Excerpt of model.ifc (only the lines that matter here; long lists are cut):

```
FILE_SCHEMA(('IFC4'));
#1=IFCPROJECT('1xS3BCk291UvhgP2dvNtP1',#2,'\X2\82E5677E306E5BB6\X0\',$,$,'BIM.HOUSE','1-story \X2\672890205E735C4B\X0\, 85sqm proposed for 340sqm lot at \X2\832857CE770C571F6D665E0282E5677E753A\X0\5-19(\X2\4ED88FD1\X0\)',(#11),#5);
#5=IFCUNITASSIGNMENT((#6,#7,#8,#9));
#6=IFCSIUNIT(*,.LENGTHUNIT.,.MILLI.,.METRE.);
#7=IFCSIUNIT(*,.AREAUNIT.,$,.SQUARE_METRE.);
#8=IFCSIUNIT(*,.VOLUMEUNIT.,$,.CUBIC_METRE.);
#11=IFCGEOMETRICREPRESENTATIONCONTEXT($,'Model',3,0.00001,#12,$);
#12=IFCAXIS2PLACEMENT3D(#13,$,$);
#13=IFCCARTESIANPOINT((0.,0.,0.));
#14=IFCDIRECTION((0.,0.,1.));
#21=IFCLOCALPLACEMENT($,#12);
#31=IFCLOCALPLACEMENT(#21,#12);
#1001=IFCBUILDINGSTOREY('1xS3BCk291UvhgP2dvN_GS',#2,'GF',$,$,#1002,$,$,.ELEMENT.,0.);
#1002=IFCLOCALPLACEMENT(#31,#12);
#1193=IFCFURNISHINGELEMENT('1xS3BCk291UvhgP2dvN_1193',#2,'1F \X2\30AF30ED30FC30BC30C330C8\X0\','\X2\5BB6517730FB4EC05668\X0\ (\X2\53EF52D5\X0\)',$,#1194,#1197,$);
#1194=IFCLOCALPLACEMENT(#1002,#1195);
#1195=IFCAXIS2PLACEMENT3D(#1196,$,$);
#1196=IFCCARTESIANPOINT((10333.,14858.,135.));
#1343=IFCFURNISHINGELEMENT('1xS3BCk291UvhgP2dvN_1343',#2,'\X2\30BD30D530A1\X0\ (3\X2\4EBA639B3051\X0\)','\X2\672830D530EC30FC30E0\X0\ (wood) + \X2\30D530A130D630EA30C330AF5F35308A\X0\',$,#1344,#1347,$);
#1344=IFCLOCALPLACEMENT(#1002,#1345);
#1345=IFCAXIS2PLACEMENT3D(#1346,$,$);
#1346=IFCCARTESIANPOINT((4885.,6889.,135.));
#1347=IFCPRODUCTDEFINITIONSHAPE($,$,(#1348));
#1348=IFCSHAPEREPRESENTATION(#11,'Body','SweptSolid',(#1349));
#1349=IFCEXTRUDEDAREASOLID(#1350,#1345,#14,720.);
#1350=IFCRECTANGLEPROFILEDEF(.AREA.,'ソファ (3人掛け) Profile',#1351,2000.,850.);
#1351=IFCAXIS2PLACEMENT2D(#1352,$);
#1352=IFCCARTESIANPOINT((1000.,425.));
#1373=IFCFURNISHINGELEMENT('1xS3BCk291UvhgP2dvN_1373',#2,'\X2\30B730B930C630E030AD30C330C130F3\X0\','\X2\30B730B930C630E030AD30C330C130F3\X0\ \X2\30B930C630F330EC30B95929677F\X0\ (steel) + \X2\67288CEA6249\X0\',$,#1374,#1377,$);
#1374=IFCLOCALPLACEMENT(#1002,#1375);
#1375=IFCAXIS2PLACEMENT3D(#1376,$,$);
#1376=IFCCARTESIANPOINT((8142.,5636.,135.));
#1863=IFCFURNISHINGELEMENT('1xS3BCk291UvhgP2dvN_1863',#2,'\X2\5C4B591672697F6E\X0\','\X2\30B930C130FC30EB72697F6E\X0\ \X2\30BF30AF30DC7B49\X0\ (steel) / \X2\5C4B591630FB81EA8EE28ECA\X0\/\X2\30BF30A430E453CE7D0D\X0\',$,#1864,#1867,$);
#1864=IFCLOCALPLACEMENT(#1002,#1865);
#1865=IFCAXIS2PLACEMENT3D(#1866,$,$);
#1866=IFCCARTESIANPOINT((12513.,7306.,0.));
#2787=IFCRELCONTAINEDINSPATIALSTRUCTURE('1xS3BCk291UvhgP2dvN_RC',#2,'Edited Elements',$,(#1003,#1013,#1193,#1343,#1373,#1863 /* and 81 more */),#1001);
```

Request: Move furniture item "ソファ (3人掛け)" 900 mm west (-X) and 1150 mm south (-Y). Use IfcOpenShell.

```python
import ifcopenshell
import ifcopenshell.api.geometry
import ifcopenshell.util.placement
import ifcopenshell.util.unit

model = ifcopenshell.open("model.ifc")
unit_scale = ifcopenshell.util.unit.calculate_unit_scale(model)

item = model.by_id(1343)
matrix = ifcopenshell.util.placement.get_local_placement(item.ObjectPlacement)
matrix[0, 3] -= 0.9 / unit_scale
matrix[1, 3] -= 1.15 / unit_scale
ifcopenshell.api.geometry.edit_object_placement(model, product=item, matrix=matrix, is_si=False)

print(ifcopenshell.util.placement.get_local_placement(item.ObjectPlacement).round(3) + 0.0)

model.write("model_edited.ifc")
```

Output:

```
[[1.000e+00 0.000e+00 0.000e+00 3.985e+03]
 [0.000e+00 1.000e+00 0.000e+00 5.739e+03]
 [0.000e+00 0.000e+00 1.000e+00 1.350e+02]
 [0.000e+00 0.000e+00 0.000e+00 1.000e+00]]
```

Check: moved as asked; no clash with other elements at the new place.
